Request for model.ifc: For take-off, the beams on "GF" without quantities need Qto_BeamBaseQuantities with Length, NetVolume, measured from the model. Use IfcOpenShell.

First a look at what the model holds.

```python
import ifcopenshell
import ifcopenshell.util.element
import ifcopenshell.util.unit

model = ifcopenshell.open("model.ifc")
print(model.schema)
for unit_type in ("LENGTHUNIT", "AREAUNIT", "VOLUMEUNIT"):
    print(unit_type, ifcopenshell.util.unit.calculate_unit_scale(model, unit_type))
storey = next(s for s in model.by_type("IfcBuildingStorey") if s.Name == "GF")
beams = [e for e in ifcopenshell.util.element.get_decomposition(storey) if e.is_a("IfcBeam")]
for e in sorted(beams, key=lambda e: e.id()):
    print(e.id(), e.is_a(), e.Name, list(ifcopenshell.util.element.get_psets(e, qtos_only=True)), sep=" | ")
```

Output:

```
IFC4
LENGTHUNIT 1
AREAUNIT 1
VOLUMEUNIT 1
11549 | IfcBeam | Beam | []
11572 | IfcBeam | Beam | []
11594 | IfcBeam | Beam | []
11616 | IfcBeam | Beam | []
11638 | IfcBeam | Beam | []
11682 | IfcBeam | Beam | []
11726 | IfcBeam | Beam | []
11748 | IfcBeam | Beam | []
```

```python
import ifcopenshell
import ifcopenshell.api.pset
import ifcopenshell.geom
import ifcopenshell.util.element
import ifcopenshell.util.shape
import ifcopenshell.util.unit

model = ifcopenshell.open("model.ifc")
unit_scale = ifcopenshell.util.unit.calculate_unit_scale(model)
volume_scale = ifcopenshell.util.unit.calculate_unit_scale(model, "VOLUMEUNIT")
settings = ifcopenshell.geom.settings()

storey = next(s for s in model.by_type("IfcBuildingStorey") if s.Name == "GF")
beams = [e for e in ifcopenshell.util.element.get_decomposition(storey) if e.is_a("IfcBeam")]

for e in sorted(beams, key=lambda e: e.id()):
    if ifcopenshell.util.element.get_psets(e, qtos_only=True, should_inherit=False):
        continue
    # Geometry comes back in metres, in the element's own axes.
    shape = ifcopenshell.geom.create_shape(settings, e)
    values = {
        "Length": ifcopenshell.util.shape.get_max_xyz(shape.geometry) / unit_scale,
        "NetVolume": ifcopenshell.util.shape.get_volume(shape.geometry) / volume_scale,
    }
    qto = ifcopenshell.api.pset.add_qto(model, product=e, name="Qto_BeamBaseQuantities")
    ifcopenshell.api.pset.edit_qto(model, qto=qto, properties=values)
    print(e.id(), {k: round(v, 3) for k, v in values.items()})

model.write("model-out.ifc")
```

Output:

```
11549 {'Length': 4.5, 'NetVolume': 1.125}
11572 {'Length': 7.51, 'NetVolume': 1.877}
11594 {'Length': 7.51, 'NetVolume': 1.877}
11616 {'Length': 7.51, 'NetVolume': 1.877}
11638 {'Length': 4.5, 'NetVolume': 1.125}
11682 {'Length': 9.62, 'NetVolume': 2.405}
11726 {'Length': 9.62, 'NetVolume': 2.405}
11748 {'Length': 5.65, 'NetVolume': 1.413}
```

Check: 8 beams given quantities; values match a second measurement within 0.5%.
